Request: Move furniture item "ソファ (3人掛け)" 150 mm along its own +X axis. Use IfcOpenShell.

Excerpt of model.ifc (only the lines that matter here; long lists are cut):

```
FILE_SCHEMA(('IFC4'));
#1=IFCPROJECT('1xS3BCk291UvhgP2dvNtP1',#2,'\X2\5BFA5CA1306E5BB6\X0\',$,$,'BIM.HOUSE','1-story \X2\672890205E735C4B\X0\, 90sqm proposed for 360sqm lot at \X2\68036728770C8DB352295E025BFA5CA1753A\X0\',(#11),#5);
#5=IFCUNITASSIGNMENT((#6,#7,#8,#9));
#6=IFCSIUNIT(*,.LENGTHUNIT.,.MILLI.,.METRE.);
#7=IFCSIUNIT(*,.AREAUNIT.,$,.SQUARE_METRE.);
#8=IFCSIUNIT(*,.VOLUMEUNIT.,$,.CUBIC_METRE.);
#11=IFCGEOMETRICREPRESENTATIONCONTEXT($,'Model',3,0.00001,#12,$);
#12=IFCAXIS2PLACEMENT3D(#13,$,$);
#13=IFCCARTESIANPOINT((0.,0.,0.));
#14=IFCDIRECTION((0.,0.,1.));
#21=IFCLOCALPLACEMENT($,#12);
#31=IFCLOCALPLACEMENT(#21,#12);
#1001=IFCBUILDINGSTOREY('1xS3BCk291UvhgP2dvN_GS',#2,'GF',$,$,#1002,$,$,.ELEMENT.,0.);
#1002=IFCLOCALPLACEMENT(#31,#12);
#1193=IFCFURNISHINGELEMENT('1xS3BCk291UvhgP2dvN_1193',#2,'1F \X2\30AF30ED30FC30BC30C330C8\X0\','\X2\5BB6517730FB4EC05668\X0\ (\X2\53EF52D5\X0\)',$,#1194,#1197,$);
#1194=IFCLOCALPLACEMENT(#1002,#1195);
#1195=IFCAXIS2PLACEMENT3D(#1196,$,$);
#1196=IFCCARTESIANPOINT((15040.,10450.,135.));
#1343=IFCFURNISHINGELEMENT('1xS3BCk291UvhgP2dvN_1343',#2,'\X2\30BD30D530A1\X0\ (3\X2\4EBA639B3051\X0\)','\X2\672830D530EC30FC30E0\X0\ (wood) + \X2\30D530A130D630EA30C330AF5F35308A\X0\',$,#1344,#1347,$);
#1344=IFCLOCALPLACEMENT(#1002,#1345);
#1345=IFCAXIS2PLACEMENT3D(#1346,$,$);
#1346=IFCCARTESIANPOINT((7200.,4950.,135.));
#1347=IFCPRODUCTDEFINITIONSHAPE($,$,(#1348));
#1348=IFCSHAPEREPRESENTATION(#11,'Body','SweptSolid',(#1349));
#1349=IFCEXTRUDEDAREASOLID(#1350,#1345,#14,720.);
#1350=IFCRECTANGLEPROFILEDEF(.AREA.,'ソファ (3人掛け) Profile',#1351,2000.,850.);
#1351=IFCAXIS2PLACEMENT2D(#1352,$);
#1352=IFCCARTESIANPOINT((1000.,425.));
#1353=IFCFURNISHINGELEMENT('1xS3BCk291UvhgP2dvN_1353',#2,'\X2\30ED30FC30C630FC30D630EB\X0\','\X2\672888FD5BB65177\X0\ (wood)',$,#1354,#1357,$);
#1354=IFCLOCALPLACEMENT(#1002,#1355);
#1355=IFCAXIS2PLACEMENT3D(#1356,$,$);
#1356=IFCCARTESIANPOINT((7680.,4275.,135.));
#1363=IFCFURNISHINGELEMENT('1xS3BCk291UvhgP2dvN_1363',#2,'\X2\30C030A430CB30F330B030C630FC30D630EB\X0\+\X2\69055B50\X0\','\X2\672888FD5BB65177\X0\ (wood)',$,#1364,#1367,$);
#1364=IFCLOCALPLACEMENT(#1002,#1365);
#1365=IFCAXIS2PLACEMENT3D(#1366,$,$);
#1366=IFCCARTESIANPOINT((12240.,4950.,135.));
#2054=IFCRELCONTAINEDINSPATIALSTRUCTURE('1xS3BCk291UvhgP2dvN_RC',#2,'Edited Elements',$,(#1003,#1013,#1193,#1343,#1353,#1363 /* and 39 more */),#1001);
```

```python
import ifcopenshell
import ifcopenshell.api.geometry
import ifcopenshell.util.placement

model = ifcopenshell.open("model.ifc")

item = model.by_guid("1xS3BCk291UvhgP2dvN_1343")
matrix = ifcopenshell.util.placement.get_local_placement(item.ObjectPlacement)
matrix[:3, 3] += matrix[:3, 0] * 150.0
ifcopenshell.api.geometry.edit_object_placement(model, product=item, matrix=matrix, is_si=False)

print(ifcopenshell.util.placement.get_local_placement(item.ObjectPlacement).round(3) + 0.0)

model.write("model_v2.ifc")
```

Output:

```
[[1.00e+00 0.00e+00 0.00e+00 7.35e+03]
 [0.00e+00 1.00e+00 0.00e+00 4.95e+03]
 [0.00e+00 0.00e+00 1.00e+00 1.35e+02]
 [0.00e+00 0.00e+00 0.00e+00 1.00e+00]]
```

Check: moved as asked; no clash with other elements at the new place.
